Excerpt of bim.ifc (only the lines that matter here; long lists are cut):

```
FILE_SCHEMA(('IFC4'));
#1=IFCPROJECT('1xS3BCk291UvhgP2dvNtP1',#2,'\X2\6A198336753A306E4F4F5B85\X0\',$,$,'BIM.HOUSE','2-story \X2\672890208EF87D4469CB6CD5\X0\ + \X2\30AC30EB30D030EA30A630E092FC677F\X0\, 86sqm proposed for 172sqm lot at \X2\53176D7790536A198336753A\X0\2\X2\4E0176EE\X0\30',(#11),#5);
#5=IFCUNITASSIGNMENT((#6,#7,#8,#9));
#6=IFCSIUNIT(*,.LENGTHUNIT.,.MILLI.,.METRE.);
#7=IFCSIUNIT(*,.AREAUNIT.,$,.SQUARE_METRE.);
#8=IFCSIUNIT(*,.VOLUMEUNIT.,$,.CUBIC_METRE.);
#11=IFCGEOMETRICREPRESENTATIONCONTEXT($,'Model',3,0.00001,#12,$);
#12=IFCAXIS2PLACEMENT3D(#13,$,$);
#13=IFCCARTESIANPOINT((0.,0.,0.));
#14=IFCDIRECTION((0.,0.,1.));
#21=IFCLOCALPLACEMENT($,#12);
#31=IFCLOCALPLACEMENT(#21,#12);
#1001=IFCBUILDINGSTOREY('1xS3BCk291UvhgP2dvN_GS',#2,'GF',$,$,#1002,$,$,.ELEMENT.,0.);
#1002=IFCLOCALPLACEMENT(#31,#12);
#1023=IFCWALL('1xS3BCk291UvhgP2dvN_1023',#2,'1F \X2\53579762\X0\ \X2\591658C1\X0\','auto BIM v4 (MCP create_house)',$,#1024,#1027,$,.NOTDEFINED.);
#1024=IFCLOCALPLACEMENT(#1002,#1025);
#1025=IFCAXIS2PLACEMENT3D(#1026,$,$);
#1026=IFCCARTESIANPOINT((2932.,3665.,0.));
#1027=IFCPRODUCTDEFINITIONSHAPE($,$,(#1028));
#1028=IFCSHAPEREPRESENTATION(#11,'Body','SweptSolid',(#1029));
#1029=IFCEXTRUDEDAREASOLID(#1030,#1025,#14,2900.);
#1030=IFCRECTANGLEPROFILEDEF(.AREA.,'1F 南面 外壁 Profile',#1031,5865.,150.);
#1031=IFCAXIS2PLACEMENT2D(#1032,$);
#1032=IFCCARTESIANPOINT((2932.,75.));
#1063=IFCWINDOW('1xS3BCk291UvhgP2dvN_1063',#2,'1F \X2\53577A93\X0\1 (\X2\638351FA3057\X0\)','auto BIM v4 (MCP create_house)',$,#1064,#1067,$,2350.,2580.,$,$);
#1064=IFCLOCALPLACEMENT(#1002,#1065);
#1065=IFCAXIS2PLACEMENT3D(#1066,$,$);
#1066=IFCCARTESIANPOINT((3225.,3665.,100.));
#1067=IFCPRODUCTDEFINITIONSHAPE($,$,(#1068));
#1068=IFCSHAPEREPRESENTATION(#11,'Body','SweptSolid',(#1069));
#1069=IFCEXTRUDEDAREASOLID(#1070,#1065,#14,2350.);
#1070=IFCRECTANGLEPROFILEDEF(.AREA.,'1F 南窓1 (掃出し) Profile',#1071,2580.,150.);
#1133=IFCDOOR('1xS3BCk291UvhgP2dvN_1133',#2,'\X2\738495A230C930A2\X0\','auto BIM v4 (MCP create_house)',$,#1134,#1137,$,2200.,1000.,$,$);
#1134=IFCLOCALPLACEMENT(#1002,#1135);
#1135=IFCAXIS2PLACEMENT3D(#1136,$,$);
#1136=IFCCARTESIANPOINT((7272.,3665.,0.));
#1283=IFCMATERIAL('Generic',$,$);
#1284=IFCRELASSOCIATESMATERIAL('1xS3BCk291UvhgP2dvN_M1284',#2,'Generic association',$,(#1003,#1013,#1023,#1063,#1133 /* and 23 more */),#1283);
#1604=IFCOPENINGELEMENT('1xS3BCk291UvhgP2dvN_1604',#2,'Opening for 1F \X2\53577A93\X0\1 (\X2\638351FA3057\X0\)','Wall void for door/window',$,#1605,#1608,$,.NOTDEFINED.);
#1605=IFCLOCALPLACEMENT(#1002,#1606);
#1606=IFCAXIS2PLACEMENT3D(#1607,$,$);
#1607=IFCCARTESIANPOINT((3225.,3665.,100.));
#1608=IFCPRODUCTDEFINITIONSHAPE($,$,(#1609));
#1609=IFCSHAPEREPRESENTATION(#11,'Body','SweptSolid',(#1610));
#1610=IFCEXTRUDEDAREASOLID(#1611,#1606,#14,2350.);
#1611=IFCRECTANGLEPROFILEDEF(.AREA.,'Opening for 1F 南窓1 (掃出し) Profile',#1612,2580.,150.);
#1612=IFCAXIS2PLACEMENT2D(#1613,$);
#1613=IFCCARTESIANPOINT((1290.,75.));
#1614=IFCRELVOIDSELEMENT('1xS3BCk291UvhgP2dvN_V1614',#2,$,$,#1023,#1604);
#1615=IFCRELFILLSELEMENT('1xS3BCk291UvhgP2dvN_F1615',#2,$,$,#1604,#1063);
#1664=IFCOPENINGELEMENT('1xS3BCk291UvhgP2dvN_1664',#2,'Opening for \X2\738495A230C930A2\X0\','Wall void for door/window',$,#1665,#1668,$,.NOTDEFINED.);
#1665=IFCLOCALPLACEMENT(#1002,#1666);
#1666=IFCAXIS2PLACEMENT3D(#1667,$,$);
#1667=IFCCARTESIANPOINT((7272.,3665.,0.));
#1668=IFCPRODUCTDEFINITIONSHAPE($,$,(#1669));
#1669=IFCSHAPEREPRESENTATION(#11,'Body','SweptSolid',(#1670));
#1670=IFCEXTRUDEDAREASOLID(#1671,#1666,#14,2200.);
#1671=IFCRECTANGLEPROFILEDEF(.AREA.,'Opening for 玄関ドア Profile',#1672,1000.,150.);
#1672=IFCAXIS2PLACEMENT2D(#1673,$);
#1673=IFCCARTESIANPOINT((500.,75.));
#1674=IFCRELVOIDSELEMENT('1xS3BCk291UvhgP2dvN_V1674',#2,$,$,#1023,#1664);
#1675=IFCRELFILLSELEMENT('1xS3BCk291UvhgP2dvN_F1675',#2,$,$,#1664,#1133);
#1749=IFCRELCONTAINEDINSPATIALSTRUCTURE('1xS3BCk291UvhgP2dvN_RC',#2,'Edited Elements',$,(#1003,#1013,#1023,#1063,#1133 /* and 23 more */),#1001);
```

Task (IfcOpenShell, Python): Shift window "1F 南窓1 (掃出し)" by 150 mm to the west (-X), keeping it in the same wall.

```python
import ifcopenshell
import ifcopenshell.api.geometry
import ifcopenshell.util.placement

model = ifcopenshell.open("bim.ifc")

window = model.by_guid("1xS3BCk291UvhgP2dvN_1063")
opening = window.FillsVoids[0].RelatingOpeningElement
wall = opening.VoidsElements[0].RelatingBuildingElement

wall_matrix = ifcopenshell.util.placement.get_local_placement(wall.ObjectPlacement)
shift = wall_matrix[:3, 0] * -150.0
before = ifcopenshell.util.placement.get_local_placement(window.ObjectPlacement)[:3, 3].copy()

# The window is not placed relative to its opening, so move both.
for product in (opening, window):
    matrix = ifcopenshell.util.placement.get_local_placement(product.ObjectPlacement)
    matrix[:3, 3] += shift
    ifcopenshell.api.geometry.edit_object_placement(model, product=product, matrix=matrix, is_si=False)

after = ifcopenshell.util.placement.get_local_placement(window.ObjectPlacement)[:3, 3]
print("window moved by", (after - before).round(3) + 0.0)

model.write("bim_rev.ifc")
```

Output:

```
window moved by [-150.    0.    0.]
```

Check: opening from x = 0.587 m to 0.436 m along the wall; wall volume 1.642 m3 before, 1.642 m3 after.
